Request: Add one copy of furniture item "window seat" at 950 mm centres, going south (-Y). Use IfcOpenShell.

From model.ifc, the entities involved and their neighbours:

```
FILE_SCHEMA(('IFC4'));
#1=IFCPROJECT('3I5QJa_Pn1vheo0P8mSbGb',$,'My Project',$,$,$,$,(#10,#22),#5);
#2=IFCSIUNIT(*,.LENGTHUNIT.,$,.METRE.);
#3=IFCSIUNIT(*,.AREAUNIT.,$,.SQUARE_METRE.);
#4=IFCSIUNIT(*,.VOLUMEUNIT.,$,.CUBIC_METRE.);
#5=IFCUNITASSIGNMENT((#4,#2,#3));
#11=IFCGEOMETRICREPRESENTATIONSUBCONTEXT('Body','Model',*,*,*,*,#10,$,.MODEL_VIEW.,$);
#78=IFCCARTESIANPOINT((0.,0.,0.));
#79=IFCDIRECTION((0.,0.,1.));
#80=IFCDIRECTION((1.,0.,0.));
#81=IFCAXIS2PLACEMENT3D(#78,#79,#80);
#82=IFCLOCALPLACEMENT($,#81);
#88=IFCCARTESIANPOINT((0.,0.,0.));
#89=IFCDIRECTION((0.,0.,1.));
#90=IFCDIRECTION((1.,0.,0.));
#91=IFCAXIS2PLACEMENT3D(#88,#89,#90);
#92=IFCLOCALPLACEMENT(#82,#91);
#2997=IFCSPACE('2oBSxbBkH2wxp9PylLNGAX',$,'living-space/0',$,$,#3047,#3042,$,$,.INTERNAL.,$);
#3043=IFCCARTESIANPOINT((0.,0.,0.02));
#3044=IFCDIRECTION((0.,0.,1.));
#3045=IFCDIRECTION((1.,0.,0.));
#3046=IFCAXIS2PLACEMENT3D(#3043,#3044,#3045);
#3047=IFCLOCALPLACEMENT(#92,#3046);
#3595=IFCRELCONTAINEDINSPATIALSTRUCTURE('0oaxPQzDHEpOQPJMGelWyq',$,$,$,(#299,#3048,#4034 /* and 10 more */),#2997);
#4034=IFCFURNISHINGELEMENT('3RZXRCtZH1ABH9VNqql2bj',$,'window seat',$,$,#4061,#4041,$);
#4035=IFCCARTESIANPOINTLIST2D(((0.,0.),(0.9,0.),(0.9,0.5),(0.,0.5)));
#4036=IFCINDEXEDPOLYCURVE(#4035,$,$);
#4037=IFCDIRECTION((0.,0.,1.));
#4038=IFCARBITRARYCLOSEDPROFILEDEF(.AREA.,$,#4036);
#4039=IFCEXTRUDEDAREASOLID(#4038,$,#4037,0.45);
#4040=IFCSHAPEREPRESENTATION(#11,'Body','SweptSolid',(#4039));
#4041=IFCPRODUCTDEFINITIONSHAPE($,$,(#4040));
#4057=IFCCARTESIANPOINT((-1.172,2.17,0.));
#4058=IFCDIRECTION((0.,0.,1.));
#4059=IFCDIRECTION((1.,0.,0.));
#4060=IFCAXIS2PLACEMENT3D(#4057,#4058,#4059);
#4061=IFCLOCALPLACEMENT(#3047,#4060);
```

```python
import numpy as np
import ifcopenshell
import ifcopenshell.api.geometry
import ifcopenshell.api.root
import ifcopenshell.util.element
import ifcopenshell.util.placement
import ifcopenshell.util.unit

model = ifcopenshell.open("model.ifc")
unit_scale = ifcopenshell.util.unit.calculate_unit_scale(model)

source = model.by_id(4034)
base = ifcopenshell.util.placement.get_local_placement(source.ObjectPlacement)
step = np.array([0.0, -1.0, 0.0]) * 0.95 / unit_scale

for i in range(1, 2):
    copy = ifcopenshell.api.root.copy_class(model, product=source)
    copy.Representation = ifcopenshell.util.element.copy_deep(
        model, source.Representation, exclude=["IfcGeometricRepresentationContext", "IfcRepresentationMap"]
    )
    matrix = base.copy()
    matrix[:3, 3] += i * step
    print("added at", matrix[:3, 3].round(3) + 0.0)
    ifcopenshell.api.geometry.edit_object_placement(model, product=copy, matrix=matrix, is_si=False)

model.write("model_edited.ifc")
```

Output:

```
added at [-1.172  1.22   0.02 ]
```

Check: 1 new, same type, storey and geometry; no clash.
